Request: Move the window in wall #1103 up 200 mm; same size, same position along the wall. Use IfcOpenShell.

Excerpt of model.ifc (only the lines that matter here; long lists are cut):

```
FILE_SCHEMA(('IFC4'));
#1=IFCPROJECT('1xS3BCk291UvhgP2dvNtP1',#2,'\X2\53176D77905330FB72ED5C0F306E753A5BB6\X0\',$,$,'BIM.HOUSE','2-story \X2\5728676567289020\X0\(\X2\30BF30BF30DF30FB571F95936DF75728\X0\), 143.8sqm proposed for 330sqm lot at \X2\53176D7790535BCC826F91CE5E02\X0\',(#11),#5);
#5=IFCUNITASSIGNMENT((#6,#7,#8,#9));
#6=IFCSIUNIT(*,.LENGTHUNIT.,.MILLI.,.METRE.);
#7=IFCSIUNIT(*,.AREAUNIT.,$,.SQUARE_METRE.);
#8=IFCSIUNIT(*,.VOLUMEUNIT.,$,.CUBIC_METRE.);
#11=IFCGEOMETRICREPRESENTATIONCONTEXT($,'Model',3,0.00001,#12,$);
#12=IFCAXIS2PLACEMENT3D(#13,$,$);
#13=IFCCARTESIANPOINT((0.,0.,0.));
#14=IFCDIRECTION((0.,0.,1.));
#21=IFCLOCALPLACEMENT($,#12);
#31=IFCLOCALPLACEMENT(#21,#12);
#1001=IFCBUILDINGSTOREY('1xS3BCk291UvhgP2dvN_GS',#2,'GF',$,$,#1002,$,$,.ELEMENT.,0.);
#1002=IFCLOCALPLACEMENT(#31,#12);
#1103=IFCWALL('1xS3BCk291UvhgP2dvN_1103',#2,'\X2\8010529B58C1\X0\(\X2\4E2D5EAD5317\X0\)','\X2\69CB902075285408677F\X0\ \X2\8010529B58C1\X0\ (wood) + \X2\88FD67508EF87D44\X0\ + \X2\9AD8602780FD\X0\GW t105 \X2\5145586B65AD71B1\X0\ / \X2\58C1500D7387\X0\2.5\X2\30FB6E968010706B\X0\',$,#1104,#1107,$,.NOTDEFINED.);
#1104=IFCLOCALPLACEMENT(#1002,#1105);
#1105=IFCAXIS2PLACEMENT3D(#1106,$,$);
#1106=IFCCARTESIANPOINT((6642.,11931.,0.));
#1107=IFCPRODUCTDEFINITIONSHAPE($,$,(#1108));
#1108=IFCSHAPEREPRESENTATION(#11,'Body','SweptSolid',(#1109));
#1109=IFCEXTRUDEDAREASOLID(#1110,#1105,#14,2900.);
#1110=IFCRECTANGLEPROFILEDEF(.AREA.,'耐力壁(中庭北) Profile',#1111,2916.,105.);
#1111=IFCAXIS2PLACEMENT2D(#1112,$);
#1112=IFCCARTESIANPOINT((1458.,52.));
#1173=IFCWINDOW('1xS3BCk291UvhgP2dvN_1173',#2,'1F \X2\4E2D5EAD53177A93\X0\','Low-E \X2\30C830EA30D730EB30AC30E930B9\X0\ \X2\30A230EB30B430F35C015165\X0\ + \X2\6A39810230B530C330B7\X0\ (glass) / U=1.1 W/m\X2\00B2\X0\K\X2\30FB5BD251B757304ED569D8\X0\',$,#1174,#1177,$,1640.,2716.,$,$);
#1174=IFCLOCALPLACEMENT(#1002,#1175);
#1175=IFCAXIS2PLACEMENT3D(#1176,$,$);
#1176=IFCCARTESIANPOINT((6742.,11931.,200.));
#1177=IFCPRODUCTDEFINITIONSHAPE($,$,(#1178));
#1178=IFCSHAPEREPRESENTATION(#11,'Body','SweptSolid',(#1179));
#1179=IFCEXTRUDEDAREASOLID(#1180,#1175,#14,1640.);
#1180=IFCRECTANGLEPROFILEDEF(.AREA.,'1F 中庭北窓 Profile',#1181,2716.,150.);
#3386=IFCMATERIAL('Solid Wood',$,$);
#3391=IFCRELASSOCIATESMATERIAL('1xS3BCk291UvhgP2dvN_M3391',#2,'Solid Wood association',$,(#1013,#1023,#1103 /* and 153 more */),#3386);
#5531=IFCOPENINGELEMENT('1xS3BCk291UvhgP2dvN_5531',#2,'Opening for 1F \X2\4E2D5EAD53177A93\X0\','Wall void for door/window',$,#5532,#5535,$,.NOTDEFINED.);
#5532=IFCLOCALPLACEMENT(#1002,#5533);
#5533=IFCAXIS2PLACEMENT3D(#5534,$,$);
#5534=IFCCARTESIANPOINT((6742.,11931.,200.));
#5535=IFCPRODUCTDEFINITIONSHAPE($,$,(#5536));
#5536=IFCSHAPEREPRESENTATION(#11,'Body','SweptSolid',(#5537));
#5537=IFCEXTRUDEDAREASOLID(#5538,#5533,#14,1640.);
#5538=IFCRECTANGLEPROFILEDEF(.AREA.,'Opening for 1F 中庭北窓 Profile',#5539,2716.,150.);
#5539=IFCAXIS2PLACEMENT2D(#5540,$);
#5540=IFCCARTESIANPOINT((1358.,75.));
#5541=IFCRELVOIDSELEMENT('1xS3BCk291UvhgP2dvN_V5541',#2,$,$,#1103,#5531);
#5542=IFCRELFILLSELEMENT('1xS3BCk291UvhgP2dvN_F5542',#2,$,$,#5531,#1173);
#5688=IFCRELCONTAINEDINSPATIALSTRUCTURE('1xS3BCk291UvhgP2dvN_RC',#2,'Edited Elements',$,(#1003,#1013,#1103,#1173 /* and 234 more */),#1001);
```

```python
import numpy as np
import ifcopenshell
import ifcopenshell.api.geometry
import ifcopenshell.util.placement
import ifcopenshell.util.unit

model = ifcopenshell.open("model.ifc")
unit_scale = ifcopenshell.util.unit.calculate_unit_scale(model)

window = model.by_guid("1xS3BCk291UvhgP2dvN_1173")
opening = window.FillsVoids[0].RelatingOpeningElement
dz = 200.0

shift = np.array([0.0, 0.0, dz])
# The window is not placed relative to its opening, so move both.
for product in (opening, window):
    matrix = ifcopenshell.util.placement.get_local_placement(product.ObjectPlacement)
    matrix[:3, 3] += shift
    ifcopenshell.api.geometry.edit_object_placement(model, product=product, matrix=matrix, is_si=False)

print(f"moved by {dz * unit_scale:+.3f} m")

model.write("model_updated.ifc")
```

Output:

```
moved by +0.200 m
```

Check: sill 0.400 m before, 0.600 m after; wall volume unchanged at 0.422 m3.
